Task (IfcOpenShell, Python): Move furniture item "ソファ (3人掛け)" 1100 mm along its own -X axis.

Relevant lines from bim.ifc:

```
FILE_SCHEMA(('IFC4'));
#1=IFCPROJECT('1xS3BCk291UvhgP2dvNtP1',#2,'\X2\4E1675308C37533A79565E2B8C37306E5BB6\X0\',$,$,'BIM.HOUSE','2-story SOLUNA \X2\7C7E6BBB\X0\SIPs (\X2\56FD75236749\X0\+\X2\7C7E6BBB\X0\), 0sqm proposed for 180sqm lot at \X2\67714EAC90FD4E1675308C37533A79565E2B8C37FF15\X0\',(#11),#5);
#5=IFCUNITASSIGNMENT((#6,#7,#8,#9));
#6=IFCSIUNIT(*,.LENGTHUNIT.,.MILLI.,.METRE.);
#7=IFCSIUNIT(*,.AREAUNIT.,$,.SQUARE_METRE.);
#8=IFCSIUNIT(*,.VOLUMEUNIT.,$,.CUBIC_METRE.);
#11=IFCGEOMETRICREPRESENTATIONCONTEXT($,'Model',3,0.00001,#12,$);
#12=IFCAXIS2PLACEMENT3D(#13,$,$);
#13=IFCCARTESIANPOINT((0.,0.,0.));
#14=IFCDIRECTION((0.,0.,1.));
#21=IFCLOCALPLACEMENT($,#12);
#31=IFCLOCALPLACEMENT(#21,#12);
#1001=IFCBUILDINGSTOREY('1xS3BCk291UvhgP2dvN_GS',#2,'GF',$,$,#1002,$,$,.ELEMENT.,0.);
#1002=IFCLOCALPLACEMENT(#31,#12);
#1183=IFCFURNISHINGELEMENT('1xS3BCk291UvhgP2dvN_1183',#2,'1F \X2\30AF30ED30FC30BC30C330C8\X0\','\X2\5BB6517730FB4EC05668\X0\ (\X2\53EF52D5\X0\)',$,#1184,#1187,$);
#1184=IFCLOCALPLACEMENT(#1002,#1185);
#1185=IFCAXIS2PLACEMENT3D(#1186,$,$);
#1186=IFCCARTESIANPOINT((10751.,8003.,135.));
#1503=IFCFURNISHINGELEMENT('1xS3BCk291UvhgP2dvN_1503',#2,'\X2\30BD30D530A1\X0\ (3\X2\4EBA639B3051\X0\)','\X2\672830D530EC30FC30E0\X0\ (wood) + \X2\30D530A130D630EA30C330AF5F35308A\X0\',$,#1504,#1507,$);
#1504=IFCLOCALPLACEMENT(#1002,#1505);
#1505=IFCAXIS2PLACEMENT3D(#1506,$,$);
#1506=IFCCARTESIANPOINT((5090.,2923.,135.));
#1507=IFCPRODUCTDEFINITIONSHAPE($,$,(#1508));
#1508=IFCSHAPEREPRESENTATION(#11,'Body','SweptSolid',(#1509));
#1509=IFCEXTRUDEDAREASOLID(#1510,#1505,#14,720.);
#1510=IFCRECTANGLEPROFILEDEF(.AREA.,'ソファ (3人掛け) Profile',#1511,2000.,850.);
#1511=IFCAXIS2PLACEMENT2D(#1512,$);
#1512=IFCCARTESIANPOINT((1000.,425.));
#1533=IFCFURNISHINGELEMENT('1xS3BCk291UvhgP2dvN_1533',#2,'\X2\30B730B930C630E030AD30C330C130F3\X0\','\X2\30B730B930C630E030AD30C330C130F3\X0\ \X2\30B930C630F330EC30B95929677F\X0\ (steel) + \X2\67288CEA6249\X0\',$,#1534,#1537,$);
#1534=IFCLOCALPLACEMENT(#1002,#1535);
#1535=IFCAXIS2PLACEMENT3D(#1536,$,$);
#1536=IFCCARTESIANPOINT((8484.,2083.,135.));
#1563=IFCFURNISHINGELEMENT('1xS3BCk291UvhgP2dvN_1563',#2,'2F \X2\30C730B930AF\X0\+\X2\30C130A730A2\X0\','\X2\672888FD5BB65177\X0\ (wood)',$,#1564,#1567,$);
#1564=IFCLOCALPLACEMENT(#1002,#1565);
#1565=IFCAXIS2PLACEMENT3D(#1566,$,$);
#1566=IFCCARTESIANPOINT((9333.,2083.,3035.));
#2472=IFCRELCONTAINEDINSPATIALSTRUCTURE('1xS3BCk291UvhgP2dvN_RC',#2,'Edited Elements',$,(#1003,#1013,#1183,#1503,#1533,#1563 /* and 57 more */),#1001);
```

```python
import ifcopenshell
import ifcopenshell.api.geometry
import ifcopenshell.util.placement
import ifcopenshell.util.unit

model = ifcopenshell.open("bim.ifc")
unit_scale = ifcopenshell.util.unit.calculate_unit_scale(model)

item = model.by_id(1503)
matrix = ifcopenshell.util.placement.get_local_placement(item.ObjectPlacement)
matrix[:3, 3] -= matrix[:3, 0] * 1.1 / unit_scale
ifcopenshell.api.geometry.edit_object_placement(model, product=item, matrix=matrix, is_si=False)

print(ifcopenshell.util.placement.get_local_placement(item.ObjectPlacement).round(3) + 0.0)

model.write("bim_v2.ifc")
```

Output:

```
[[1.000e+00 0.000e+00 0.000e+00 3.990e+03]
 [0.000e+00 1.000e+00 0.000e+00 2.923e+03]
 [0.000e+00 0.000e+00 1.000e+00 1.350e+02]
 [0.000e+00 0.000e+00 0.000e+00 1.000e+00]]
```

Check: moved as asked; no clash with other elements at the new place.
